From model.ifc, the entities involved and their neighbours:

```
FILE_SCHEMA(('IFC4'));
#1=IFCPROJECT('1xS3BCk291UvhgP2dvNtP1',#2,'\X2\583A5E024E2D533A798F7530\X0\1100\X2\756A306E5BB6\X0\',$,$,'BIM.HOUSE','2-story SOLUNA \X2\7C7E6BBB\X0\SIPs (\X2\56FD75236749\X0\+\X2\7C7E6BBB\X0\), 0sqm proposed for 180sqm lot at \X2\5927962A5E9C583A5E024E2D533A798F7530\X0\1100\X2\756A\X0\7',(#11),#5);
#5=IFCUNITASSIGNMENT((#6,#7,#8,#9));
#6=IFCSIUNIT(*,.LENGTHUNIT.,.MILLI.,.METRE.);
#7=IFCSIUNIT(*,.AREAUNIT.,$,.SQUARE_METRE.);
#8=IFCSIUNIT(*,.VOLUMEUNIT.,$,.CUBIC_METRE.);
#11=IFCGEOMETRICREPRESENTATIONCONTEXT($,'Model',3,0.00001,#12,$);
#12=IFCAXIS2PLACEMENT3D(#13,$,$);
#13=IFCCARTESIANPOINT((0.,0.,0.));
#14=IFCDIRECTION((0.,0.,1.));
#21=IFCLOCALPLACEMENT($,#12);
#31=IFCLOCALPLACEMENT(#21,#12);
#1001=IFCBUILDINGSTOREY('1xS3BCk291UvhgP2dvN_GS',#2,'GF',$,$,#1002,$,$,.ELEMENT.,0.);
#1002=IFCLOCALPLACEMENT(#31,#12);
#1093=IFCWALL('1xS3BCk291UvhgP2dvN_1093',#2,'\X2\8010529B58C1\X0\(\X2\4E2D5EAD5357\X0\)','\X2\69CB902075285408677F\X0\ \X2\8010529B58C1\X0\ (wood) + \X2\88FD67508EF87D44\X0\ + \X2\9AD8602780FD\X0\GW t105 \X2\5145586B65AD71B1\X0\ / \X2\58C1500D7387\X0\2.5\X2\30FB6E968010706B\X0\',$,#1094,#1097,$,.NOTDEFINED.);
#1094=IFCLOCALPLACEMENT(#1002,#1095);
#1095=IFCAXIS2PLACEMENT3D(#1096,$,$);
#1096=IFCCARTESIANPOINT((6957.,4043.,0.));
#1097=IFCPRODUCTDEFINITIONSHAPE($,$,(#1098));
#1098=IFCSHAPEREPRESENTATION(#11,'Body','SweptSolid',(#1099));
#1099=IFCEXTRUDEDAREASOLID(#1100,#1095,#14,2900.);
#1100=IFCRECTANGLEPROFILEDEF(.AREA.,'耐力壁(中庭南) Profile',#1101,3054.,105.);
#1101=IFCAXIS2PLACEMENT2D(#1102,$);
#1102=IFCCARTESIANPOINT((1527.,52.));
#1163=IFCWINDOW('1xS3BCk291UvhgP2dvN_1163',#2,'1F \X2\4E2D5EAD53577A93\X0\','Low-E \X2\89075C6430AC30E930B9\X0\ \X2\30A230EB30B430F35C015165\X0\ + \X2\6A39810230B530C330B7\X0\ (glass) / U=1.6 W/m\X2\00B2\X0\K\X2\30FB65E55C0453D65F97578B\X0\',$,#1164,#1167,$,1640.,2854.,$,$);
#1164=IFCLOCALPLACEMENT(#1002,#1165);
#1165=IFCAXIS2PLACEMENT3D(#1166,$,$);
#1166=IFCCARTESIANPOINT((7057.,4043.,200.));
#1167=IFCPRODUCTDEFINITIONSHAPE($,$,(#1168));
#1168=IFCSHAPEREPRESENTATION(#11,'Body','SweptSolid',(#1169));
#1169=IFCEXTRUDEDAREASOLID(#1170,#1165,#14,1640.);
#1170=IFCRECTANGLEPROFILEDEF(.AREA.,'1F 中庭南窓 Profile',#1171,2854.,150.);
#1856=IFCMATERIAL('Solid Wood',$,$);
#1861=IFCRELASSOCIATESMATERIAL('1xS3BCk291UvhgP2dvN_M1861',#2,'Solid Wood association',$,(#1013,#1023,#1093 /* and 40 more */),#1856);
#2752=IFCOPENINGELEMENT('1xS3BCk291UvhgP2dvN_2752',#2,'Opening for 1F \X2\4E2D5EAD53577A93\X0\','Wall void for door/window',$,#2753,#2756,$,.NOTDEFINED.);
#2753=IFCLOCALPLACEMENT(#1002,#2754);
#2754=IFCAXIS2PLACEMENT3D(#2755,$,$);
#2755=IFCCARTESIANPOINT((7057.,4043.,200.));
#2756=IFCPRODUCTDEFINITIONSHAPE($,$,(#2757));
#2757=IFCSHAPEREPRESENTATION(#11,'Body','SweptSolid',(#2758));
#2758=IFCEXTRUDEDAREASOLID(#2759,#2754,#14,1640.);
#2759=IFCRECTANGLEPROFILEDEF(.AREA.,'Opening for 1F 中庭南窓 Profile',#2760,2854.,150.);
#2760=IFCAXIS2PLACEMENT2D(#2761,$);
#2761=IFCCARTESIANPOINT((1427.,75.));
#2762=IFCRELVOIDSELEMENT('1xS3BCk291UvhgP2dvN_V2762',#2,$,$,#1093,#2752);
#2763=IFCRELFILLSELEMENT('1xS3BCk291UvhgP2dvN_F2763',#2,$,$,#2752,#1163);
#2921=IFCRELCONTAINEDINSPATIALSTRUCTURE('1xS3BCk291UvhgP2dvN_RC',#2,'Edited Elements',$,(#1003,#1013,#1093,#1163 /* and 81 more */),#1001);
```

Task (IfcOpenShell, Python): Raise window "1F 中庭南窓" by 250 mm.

```python
import numpy as np
import ifcopenshell
import ifcopenshell.api.geometry
import ifcopenshell.util.placement
import ifcopenshell.util.unit

model = ifcopenshell.open("model.ifc")
unit_scale = ifcopenshell.util.unit.calculate_unit_scale(model)

window = model.by_id(1163)
opening = window.FillsVoids[0].RelatingOpeningElement
dz = 0.25 / unit_scale

shift = np.array([0.0, 0.0, dz])
# The window is not placed relative to its opening, so move both.
for product in (opening, window):
    matrix = ifcopenshell.util.placement.get_local_placement(product.ObjectPlacement)
    matrix[:3, 3] += shift
    ifcopenshell.api.geometry.edit_object_placement(model, product=product, matrix=matrix, is_si=False)

print(f"moved by {dz * unit_scale:+.3f} m")

model.write("model_v2.ifc")
```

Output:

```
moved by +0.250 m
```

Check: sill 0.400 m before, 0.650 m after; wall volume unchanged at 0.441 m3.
